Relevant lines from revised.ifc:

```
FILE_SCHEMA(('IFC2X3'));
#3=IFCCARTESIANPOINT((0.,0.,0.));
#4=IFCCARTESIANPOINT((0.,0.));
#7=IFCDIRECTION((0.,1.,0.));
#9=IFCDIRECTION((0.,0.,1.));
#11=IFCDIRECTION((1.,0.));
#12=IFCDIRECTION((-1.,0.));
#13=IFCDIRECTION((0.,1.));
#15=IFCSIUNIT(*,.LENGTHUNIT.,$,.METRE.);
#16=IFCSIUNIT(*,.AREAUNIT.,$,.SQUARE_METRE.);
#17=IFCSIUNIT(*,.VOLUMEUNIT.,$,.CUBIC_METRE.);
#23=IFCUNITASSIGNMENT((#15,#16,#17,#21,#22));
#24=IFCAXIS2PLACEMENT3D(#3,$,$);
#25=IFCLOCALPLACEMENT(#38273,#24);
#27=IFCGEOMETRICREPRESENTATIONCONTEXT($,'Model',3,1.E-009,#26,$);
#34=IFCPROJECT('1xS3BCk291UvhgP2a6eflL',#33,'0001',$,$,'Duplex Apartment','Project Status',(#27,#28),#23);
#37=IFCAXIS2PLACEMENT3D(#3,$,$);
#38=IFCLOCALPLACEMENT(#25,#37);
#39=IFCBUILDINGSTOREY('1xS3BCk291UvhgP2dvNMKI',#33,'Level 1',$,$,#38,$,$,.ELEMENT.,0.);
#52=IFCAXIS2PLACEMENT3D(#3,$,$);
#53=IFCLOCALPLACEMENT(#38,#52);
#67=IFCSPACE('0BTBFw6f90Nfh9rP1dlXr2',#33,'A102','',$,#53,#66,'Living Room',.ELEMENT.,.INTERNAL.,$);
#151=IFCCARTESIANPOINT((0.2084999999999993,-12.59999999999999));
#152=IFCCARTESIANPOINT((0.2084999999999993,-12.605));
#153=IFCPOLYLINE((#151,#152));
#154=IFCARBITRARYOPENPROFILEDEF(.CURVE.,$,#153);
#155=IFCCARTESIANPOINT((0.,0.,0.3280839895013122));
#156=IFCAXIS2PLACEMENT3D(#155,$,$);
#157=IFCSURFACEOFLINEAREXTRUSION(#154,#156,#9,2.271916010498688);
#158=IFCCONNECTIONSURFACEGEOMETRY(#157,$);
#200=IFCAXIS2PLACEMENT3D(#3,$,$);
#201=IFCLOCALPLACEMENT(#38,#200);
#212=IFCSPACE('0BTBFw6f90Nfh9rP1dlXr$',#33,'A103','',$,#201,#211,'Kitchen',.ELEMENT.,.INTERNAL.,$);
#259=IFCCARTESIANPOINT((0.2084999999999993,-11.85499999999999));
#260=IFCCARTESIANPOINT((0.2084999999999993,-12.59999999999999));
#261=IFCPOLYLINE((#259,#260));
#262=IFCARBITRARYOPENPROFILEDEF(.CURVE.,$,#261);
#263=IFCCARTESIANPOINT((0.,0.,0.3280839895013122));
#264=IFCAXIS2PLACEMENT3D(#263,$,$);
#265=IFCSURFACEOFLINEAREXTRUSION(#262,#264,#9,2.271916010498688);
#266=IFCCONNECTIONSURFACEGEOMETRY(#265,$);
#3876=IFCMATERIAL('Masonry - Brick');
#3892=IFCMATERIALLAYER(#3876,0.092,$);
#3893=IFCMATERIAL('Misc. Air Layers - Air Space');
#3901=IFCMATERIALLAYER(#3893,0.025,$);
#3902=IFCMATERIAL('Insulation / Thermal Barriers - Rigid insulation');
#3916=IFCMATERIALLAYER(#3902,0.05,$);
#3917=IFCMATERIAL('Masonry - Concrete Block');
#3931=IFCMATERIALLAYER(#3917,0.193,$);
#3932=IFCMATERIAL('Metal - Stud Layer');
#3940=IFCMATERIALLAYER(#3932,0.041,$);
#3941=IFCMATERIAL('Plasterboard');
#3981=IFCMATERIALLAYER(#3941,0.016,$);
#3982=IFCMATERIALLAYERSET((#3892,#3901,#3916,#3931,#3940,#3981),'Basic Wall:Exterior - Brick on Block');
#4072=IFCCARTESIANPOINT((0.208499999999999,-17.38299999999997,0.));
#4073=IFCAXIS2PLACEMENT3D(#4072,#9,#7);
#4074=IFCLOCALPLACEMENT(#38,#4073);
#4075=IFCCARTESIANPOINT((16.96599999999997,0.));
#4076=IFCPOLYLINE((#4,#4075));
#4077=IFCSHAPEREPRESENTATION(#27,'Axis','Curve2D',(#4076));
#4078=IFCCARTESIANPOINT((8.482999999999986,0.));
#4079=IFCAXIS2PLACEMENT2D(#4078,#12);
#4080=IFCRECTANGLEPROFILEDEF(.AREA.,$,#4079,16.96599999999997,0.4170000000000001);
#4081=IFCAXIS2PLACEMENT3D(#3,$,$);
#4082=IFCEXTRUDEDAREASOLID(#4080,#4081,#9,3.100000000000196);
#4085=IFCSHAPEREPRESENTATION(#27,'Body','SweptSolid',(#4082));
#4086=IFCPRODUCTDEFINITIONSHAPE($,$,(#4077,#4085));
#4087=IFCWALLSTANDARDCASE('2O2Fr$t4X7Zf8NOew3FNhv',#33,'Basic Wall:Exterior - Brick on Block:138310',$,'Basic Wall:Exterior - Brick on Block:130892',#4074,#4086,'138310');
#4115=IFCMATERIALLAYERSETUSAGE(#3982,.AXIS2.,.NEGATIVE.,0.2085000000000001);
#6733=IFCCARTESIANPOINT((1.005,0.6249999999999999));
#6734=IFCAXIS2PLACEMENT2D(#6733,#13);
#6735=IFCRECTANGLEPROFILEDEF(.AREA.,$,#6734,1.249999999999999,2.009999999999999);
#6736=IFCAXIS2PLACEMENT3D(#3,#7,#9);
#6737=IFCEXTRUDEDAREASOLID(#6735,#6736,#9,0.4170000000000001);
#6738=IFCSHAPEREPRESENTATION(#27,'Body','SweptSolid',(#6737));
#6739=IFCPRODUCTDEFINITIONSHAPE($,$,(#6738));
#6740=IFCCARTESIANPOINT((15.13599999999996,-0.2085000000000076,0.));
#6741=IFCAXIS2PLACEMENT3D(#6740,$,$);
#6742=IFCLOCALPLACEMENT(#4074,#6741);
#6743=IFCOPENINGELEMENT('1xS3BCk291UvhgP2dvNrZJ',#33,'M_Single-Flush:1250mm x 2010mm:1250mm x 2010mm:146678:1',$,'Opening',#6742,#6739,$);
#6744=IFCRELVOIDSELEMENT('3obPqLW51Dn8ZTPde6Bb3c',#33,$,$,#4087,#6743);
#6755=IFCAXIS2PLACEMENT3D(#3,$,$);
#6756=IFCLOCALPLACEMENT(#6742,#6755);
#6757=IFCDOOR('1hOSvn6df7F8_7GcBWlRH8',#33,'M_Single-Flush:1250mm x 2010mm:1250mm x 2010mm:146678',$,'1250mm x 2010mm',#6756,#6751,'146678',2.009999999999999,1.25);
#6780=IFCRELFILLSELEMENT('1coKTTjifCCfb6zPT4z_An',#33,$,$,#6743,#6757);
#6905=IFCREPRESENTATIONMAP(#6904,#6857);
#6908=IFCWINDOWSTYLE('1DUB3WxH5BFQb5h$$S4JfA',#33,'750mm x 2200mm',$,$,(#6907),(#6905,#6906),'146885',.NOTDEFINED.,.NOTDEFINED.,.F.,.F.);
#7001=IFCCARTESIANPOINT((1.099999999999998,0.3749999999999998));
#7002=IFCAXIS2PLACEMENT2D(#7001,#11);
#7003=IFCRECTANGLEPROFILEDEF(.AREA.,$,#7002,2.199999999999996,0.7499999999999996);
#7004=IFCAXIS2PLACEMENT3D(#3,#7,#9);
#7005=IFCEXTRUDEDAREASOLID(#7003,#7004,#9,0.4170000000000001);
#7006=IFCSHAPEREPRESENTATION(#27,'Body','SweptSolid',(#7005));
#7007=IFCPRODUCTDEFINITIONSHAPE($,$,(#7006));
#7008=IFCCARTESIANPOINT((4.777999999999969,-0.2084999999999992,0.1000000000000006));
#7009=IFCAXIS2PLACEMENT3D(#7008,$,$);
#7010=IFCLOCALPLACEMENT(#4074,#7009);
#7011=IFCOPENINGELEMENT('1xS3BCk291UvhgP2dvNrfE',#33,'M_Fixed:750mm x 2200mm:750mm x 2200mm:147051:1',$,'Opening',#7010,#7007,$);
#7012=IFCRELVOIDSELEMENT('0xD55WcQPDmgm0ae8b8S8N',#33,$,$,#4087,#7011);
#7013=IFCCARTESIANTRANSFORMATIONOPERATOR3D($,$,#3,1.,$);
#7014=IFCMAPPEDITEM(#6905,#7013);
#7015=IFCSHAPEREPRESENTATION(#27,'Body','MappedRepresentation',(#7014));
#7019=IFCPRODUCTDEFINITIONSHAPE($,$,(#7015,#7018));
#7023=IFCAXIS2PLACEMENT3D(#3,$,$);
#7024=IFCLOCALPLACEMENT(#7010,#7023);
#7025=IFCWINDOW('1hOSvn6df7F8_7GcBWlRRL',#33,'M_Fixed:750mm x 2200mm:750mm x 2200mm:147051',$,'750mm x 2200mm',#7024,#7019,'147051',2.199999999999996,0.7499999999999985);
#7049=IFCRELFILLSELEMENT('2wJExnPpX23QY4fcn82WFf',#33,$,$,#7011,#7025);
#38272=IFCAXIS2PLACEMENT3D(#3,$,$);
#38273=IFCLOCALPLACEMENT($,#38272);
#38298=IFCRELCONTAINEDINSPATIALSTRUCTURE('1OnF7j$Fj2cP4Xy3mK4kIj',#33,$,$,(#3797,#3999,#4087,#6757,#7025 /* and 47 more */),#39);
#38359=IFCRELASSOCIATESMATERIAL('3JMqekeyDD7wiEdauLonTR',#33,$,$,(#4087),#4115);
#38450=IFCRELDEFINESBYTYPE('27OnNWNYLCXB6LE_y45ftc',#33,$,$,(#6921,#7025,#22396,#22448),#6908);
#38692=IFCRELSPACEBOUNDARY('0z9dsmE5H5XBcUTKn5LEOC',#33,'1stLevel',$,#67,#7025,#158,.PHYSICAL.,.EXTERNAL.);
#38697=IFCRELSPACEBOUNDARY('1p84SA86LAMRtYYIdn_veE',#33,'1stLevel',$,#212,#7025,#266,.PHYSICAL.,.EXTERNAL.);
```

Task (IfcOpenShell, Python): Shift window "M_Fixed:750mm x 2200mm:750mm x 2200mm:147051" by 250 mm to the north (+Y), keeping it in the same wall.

```python
import numpy as np
import ifcopenshell
import ifcopenshell.api.geometry
import ifcopenshell.util.placement
import ifcopenshell.util.unit

model = ifcopenshell.open("revised.ifc")
unit_scale = ifcopenshell.util.unit.calculate_unit_scale(model)

window = model.by_guid("1hOSvn6df7F8_7GcBWlRRL")
opening = window.FillsVoids[0].RelatingOpeningElement
wall = opening.VoidsElements[0].RelatingBuildingElement

wall_matrix = ifcopenshell.util.placement.get_local_placement(wall.ObjectPlacement)
shift = wall_matrix[:3, 0] * 0.25 / unit_scale
before = ifcopenshell.util.placement.get_local_placement(window.ObjectPlacement)[:3, 3].copy()

# The window is placed relative to its opening, so it follows when the opening moves.
matrix = ifcopenshell.util.placement.get_local_placement(opening.ObjectPlacement)
matrix[:3, 3] += shift
ifcopenshell.api.geometry.edit_object_placement(
    model, product=opening, matrix=matrix, is_si=False, should_transform_children=True
)

# Space boundary surfaces are stored in each space's coordinates; move them too.
for rel in window.ProvidesBoundaries:
    if not rel.ConnectionGeometry:
        continue
    surface = rel.ConnectionGeometry.SurfaceOnRelatingElement
    space_matrix = ifcopenshell.util.placement.get_local_placement(rel.RelatingSpace.ObjectPlacement)
    point = np.array(surface.Position.Location.Coordinates) + space_matrix[:3, :3].T @ shift
    surface.Position = model.createIfcAxis2Placement3D(
        model.createIfcCartesianPoint(point.tolist()), surface.Position.Axis, surface.Position.RefDirection
    )

after = ifcopenshell.util.placement.get_local_placement(window.ObjectPlacement)[:3, 3]
print("window moved by", (after - before).round(3) + 0.0)

model.write("revised_edited.ifc")
```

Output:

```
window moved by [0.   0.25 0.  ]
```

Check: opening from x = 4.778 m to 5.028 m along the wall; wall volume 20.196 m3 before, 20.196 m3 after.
